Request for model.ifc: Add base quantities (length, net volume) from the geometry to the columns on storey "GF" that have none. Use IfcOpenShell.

First a look at what the model holds.

```python
import ifcopenshell
import ifcopenshell.util.element
import ifcopenshell.util.unit

model = ifcopenshell.open("model.ifc")
print(model.schema)
for unit_type in ("LENGTHUNIT", "AREAUNIT", "VOLUMEUNIT"):
    print(unit_type, ifcopenshell.util.unit.calculate_unit_scale(model, unit_type))
storey = next(s for s in model.by_type("IfcBuildingStorey") if s.Name == "GF")
columns = [e for e in ifcopenshell.util.element.get_decomposition(storey) if e.is_a("IfcColumn")]
for e in sorted(columns, key=lambda e: e.id()):
    print(e.id(), e.is_a(), e.Name, list(ifcopenshell.util.element.get_psets(e, qtos_only=True)), sep=" | ")
```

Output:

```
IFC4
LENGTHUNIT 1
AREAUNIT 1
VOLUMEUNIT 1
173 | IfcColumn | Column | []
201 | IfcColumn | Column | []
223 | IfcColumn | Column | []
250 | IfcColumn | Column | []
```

```python
import ifcopenshell
import ifcopenshell.api.pset
import ifcopenshell.geom
import ifcopenshell.util.element
import ifcopenshell.util.shape
import ifcopenshell.util.unit

model = ifcopenshell.open("model.ifc")
unit_scale = ifcopenshell.util.unit.calculate_unit_scale(model)
volume_scale = ifcopenshell.util.unit.calculate_unit_scale(model, "VOLUMEUNIT")
settings = ifcopenshell.geom.settings()

storey = next(s for s in model.by_type("IfcBuildingStorey") if s.Name == "GF")
columns = [e for e in ifcopenshell.util.element.get_decomposition(storey) if e.is_a("IfcColumn")]

for e in sorted(columns, key=lambda e: e.id()):
    if ifcopenshell.util.element.get_psets(e, qtos_only=True, should_inherit=False):
        continue
    # Geometry comes back in metres, in the element's own axes.
    shape = ifcopenshell.geom.create_shape(settings, e)
    values = {
        "Length": ifcopenshell.util.shape.get_z(shape.geometry) / unit_scale,
        "NetVolume": ifcopenshell.util.shape.get_volume(shape.geometry) / volume_scale,
    }
    qto = ifcopenshell.api.pset.add_qto(model, product=e, name="Qto_ColumnBaseQuantities")
    ifcopenshell.api.pset.edit_qto(model, qto=qto, properties=values)
    print(e.id(), {k: round(v, 3) for k, v in values.items()})

model.write("model-out.ifc")
```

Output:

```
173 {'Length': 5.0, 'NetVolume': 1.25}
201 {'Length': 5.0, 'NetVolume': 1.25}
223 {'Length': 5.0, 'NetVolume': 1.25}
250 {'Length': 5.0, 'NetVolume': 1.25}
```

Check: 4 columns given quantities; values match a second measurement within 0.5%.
